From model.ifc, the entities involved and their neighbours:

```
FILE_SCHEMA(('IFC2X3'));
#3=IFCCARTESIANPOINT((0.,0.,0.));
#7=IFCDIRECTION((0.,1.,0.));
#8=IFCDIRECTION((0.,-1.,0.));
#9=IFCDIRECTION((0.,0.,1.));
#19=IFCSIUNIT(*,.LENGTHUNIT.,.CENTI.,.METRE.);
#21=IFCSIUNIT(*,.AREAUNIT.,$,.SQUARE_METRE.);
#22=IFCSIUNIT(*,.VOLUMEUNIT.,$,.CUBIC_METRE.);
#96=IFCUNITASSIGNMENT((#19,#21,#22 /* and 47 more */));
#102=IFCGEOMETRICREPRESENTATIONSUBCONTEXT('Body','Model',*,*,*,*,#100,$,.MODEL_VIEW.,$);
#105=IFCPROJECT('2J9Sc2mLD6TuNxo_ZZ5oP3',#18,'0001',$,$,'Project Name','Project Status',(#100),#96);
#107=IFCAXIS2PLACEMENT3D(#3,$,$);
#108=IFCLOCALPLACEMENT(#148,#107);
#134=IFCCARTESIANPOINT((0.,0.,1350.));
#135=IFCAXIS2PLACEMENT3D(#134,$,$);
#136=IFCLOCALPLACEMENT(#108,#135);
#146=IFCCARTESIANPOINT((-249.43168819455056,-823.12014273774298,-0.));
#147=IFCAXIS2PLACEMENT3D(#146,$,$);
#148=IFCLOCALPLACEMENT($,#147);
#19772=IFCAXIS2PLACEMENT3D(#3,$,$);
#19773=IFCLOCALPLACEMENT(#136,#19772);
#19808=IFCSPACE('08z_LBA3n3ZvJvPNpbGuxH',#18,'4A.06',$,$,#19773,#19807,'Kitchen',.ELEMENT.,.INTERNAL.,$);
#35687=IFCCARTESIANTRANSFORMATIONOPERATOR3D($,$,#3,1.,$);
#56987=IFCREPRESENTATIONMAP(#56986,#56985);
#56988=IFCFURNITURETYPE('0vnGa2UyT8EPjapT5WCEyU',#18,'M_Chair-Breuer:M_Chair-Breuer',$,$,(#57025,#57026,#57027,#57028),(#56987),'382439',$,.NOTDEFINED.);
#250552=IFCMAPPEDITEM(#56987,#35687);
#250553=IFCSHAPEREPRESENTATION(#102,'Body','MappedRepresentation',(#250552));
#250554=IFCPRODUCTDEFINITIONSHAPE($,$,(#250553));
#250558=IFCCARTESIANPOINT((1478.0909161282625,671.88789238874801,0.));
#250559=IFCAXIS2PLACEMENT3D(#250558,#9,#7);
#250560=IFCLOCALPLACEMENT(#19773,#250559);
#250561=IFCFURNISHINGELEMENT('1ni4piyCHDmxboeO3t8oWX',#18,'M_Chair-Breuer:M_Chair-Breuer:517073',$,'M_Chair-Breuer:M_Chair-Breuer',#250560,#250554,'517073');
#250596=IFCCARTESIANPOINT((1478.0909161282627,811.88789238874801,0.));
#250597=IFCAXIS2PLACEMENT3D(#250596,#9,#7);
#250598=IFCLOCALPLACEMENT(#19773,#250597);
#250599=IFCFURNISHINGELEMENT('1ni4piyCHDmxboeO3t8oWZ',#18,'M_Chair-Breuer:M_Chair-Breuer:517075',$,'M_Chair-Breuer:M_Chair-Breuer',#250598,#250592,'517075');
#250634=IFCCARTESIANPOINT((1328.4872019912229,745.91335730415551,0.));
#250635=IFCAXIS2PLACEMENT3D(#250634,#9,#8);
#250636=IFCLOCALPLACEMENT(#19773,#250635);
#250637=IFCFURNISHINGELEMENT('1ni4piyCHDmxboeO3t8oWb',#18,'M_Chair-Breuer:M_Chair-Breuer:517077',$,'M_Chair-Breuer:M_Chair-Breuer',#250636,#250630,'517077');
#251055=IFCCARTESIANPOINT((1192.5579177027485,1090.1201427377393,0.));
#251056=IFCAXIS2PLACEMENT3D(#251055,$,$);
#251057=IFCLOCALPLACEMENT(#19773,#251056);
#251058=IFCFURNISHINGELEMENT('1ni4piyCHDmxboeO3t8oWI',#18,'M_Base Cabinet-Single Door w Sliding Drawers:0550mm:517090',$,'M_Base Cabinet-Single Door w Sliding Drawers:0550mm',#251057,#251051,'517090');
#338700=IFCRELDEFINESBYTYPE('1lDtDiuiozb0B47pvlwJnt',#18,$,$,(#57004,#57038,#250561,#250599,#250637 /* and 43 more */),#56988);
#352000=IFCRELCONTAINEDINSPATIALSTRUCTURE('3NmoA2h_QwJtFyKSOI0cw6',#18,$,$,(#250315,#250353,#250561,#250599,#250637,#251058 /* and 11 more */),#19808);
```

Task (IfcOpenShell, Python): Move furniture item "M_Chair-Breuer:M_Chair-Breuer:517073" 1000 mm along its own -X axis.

```python
import ifcopenshell
import ifcopenshell.api.geometry
import ifcopenshell.util.placement
import ifcopenshell.util.unit

model = ifcopenshell.open("model.ifc")
unit_scale = ifcopenshell.util.unit.calculate_unit_scale(model)

item = model.by_guid("1ni4piyCHDmxboeO3t8oWX")
matrix = ifcopenshell.util.placement.get_local_placement(item.ObjectPlacement)
matrix[:3, 3] -= matrix[:3, 0] * 1 / unit_scale
ifcopenshell.api.geometry.edit_object_placement(model, product=item, matrix=matrix, is_si=False)

print(ifcopenshell.util.placement.get_local_placement(item.ObjectPlacement).round(3) + 0.0)

model.write("model_rev.ifc")
```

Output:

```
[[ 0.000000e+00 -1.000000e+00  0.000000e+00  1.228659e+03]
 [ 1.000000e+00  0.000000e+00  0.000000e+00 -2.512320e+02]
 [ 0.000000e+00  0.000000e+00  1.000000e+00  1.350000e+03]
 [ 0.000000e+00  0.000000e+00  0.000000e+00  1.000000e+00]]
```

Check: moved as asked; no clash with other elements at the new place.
